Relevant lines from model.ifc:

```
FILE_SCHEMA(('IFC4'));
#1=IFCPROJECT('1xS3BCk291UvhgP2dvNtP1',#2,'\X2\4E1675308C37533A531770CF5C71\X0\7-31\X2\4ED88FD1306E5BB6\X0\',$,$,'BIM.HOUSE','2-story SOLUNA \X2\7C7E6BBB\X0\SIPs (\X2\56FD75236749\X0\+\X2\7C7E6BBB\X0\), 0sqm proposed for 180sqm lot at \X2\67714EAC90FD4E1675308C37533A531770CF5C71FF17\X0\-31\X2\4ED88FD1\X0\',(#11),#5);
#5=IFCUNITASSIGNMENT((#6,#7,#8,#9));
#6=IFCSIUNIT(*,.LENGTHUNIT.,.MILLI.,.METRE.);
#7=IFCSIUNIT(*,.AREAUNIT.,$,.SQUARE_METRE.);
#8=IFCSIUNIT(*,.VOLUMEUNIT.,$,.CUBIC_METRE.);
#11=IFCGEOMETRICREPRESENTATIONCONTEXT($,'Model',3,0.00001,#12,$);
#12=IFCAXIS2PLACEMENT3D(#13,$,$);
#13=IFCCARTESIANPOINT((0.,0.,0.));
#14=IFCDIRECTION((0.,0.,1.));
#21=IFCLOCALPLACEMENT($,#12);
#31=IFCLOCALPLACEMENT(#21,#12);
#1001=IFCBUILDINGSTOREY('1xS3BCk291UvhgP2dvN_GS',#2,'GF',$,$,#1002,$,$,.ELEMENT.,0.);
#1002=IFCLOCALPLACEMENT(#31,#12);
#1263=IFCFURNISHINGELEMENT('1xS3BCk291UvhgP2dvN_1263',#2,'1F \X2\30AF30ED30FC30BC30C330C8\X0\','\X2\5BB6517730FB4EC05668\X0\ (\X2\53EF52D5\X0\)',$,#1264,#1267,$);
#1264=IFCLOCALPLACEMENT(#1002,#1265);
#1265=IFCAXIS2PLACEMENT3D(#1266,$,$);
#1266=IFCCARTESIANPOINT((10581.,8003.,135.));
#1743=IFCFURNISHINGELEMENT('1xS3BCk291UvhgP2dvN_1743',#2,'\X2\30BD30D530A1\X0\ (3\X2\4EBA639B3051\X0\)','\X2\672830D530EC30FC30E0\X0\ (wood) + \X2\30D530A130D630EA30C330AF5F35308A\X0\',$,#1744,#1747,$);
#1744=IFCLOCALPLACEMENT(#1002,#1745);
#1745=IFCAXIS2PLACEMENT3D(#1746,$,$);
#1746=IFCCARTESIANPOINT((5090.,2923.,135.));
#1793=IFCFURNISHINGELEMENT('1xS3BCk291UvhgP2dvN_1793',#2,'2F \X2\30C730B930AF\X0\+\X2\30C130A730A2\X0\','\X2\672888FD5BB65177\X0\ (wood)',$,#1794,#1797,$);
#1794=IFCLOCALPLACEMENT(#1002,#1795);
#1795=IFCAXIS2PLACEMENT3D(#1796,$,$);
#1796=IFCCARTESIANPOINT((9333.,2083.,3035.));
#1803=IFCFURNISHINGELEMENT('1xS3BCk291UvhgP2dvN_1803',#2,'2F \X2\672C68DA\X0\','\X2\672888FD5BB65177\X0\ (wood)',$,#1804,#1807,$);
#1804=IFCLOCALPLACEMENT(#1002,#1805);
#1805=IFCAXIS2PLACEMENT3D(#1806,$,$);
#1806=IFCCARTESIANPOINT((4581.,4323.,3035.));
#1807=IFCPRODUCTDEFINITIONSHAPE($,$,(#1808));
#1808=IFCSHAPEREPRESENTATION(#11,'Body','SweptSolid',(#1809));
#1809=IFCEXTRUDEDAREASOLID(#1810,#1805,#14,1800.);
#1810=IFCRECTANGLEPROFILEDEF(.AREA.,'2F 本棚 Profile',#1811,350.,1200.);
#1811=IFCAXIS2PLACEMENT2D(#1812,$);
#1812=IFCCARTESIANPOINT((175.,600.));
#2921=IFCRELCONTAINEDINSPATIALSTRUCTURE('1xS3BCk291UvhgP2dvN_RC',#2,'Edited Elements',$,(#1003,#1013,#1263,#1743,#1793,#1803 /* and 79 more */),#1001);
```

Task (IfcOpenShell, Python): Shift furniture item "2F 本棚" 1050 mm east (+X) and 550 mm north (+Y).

```python
import ifcopenshell
import ifcopenshell.api.geometry
import ifcopenshell.util.placement
import ifcopenshell.util.unit

model = ifcopenshell.open("model.ifc")
unit_scale = ifcopenshell.util.unit.calculate_unit_scale(model)

item = model.by_guid("1xS3BCk291UvhgP2dvN_1803")
matrix = ifcopenshell.util.placement.get_local_placement(item.ObjectPlacement)
matrix[0, 3] += 1.05 / unit_scale
matrix[1, 3] += 0.55 / unit_scale
ifcopenshell.api.geometry.edit_object_placement(model, product=item, matrix=matrix, is_si=False)

print(ifcopenshell.util.placement.get_local_placement(item.ObjectPlacement).round(3) + 0.0)

model.write("model_rev.ifc")
```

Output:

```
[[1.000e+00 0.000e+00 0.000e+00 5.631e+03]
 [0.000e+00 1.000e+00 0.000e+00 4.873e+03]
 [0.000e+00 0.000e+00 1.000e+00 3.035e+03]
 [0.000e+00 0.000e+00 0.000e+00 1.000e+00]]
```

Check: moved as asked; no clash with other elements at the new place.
